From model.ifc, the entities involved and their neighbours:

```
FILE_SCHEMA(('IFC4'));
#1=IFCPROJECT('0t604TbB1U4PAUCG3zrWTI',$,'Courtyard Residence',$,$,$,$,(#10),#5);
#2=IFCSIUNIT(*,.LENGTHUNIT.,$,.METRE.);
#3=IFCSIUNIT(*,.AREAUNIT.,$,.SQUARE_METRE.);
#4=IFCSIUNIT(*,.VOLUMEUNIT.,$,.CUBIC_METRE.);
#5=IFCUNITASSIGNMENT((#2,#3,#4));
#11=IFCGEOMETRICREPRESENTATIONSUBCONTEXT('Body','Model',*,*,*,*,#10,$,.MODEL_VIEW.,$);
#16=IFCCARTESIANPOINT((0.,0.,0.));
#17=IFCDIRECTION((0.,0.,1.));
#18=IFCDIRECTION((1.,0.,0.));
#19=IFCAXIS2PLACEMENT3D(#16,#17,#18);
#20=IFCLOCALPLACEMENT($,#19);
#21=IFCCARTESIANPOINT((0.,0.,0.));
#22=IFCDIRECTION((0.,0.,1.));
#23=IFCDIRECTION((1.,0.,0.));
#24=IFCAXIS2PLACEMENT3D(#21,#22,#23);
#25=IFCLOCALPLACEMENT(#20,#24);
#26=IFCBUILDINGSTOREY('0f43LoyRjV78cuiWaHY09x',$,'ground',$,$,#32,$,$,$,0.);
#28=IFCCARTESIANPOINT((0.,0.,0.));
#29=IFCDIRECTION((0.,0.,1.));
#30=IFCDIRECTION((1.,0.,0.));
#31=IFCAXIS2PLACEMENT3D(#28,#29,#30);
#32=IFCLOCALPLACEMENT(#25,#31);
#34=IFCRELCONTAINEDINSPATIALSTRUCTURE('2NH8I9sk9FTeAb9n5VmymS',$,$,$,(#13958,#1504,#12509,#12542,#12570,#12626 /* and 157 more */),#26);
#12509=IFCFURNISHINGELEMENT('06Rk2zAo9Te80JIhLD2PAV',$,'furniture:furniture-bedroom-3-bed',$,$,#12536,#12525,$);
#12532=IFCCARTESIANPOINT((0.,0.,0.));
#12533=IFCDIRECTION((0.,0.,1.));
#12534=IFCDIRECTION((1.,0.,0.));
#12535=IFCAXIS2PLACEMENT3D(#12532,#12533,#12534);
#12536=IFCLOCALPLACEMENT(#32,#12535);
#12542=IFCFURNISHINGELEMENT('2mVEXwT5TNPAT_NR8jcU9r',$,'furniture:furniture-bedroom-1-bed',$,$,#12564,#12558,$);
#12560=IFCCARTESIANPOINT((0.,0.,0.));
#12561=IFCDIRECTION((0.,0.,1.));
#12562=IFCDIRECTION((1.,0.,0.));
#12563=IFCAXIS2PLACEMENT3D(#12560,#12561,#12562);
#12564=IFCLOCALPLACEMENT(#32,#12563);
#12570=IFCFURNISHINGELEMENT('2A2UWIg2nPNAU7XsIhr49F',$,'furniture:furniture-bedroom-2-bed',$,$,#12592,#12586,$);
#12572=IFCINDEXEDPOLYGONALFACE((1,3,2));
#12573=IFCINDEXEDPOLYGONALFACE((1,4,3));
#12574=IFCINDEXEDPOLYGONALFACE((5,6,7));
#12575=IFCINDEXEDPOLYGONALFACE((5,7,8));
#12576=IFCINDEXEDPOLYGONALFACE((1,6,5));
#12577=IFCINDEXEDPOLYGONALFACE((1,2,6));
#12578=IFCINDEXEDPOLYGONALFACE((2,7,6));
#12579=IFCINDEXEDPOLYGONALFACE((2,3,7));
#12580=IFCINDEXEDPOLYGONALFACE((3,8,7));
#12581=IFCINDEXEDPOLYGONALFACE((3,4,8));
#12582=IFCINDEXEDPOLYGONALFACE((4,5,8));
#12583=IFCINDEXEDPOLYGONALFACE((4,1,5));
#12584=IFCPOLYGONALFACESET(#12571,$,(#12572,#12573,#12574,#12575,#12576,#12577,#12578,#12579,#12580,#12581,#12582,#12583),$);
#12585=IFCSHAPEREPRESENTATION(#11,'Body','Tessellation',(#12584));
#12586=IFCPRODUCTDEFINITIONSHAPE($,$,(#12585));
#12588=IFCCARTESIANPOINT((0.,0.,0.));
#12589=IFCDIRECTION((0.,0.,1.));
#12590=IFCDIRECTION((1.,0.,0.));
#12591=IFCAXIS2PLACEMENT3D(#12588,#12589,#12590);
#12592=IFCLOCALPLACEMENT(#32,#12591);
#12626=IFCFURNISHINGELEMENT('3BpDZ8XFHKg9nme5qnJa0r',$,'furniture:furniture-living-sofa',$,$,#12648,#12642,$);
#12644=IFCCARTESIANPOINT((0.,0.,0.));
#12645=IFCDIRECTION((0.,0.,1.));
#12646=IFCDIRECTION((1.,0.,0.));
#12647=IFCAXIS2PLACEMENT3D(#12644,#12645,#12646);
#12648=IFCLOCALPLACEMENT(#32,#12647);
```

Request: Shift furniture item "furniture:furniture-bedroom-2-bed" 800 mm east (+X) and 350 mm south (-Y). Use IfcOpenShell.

```python
import ifcopenshell
import ifcopenshell.api.geometry
import ifcopenshell.util.placement

model = ifcopenshell.open("model.ifc")

item = model.by_guid("2A2UWIg2nPNAU7XsIhr49F")
matrix = ifcopenshell.util.placement.get_local_placement(item.ObjectPlacement)
matrix[0, 3] += 0.8
matrix[1, 3] -= 0.35
ifcopenshell.api.geometry.edit_object_placement(model, product=item, matrix=matrix, is_si=False)

print(ifcopenshell.util.placement.get_local_placement(item.ObjectPlacement).round(3) + 0.0)

model.write("model_rev.ifc")
```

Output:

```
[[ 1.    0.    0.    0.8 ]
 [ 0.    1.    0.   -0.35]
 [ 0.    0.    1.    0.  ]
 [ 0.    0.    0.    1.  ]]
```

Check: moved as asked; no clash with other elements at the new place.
